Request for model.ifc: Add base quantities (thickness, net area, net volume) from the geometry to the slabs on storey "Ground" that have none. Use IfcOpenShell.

First a look at what the model holds.

```python
import ifcopenshell
import ifcopenshell.util.element
import ifcopenshell.util.unit

model = ifcopenshell.open("model.ifc")
print(model.schema)
for unit_type in ("LENGTHUNIT", "AREAUNIT", "VOLUMEUNIT"):
    print(unit_type, ifcopenshell.util.unit.calculate_unit_scale(model, unit_type))
storey = next(s for s in model.by_type("IfcBuildingStorey") if s.Name == "Ground")
slabs = [e for e in ifcopenshell.util.element.get_decomposition(storey) if e.is_a("IfcSlab")]
for e in sorted(slabs, key=lambda e: e.id()):
    print(e.id(), e.is_a(), e.Name, list(ifcopenshell.util.element.get_psets(e, qtos_only=True)), sep=" | ")
```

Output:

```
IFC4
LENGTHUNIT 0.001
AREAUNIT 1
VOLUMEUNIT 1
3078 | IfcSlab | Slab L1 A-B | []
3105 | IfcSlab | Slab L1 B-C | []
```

```python
import ifcopenshell
import ifcopenshell.api.pset
import ifcopenshell.geom
import ifcopenshell.util.element
import ifcopenshell.util.shape
import ifcopenshell.util.unit

model = ifcopenshell.open("model.ifc")
unit_scale = ifcopenshell.util.unit.calculate_unit_scale(model)
area_scale = ifcopenshell.util.unit.calculate_unit_scale(model, "AREAUNIT")
volume_scale = ifcopenshell.util.unit.calculate_unit_scale(model, "VOLUMEUNIT")
settings = ifcopenshell.geom.settings()

storey = next(s for s in model.by_type("IfcBuildingStorey") if s.Name == "Ground")
slabs = [e for e in ifcopenshell.util.element.get_decomposition(storey) if e.is_a("IfcSlab")]

for e in sorted(slabs, key=lambda e: e.id()):
    if ifcopenshell.util.element.get_psets(e, qtos_only=True, should_inherit=False):
        continue
    # Geometry comes back in metres, in the element's own axes.
    shape = ifcopenshell.geom.create_shape(settings, e)
    values = {
        "Width": ifcopenshell.util.shape.get_z(shape.geometry) / unit_scale,
        "NetArea": ifcopenshell.util.shape.get_footprint_area(shape.geometry) / area_scale,
        "NetVolume": ifcopenshell.util.shape.get_volume(shape.geometry) / volume_scale,
    }
    qto = ifcopenshell.api.pset.add_qto(model, product=e, name="Qto_SlabBaseQuantities")
    ifcopenshell.api.pset.edit_qto(model, qto=qto, properties=values)
    print(e.id(), {k: round(v, 3) for k, v in values.items()})

model.write("model_updated.ifc")
```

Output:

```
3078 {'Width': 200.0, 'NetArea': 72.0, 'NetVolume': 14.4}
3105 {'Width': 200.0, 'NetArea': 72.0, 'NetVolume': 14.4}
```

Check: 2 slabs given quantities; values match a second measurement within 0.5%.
